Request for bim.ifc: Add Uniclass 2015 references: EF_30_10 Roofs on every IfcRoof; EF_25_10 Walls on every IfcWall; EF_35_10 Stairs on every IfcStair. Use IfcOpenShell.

First a look at what the model holds.

```python
import ifcopenshell

model = ifcopenshell.open("bim.ifc")
print(model.schema)
print("classifications:", [c.Name for c in model.by_type("IfcClassification")])
for ifc_class in ("IfcDoor", "IfcRoof", "IfcStair", "IfcWall", "IfcWindow"):
    print(ifc_class, len(model.by_type(ifc_class)))
```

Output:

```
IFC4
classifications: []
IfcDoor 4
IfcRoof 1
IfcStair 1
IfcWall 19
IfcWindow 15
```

```python
import ifcopenshell
import ifcopenshell.api.classification

model = ifcopenshell.open("bim.ifc")

system = ifcopenshell.api.classification.add_classification(model, classification="Uniclass 2015")

codes = {
    "IfcRoof": ("EF_30_10", "Roofs"),
    "IfcWall": ("EF_25_10", "Walls"),
    "IfcStair": ("EF_35_10", "Stairs"),
}
for ifc_class, (code, name) in codes.items():
    products = model.by_type(ifc_class)
    ifcopenshell.api.classification.add_reference(
        model, products=products, classification=system, identification=code, name=name
    )
    print(code, len(products))

model.write("bim_rev.ifc")
```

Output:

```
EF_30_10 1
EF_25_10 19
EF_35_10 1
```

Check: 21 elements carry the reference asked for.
